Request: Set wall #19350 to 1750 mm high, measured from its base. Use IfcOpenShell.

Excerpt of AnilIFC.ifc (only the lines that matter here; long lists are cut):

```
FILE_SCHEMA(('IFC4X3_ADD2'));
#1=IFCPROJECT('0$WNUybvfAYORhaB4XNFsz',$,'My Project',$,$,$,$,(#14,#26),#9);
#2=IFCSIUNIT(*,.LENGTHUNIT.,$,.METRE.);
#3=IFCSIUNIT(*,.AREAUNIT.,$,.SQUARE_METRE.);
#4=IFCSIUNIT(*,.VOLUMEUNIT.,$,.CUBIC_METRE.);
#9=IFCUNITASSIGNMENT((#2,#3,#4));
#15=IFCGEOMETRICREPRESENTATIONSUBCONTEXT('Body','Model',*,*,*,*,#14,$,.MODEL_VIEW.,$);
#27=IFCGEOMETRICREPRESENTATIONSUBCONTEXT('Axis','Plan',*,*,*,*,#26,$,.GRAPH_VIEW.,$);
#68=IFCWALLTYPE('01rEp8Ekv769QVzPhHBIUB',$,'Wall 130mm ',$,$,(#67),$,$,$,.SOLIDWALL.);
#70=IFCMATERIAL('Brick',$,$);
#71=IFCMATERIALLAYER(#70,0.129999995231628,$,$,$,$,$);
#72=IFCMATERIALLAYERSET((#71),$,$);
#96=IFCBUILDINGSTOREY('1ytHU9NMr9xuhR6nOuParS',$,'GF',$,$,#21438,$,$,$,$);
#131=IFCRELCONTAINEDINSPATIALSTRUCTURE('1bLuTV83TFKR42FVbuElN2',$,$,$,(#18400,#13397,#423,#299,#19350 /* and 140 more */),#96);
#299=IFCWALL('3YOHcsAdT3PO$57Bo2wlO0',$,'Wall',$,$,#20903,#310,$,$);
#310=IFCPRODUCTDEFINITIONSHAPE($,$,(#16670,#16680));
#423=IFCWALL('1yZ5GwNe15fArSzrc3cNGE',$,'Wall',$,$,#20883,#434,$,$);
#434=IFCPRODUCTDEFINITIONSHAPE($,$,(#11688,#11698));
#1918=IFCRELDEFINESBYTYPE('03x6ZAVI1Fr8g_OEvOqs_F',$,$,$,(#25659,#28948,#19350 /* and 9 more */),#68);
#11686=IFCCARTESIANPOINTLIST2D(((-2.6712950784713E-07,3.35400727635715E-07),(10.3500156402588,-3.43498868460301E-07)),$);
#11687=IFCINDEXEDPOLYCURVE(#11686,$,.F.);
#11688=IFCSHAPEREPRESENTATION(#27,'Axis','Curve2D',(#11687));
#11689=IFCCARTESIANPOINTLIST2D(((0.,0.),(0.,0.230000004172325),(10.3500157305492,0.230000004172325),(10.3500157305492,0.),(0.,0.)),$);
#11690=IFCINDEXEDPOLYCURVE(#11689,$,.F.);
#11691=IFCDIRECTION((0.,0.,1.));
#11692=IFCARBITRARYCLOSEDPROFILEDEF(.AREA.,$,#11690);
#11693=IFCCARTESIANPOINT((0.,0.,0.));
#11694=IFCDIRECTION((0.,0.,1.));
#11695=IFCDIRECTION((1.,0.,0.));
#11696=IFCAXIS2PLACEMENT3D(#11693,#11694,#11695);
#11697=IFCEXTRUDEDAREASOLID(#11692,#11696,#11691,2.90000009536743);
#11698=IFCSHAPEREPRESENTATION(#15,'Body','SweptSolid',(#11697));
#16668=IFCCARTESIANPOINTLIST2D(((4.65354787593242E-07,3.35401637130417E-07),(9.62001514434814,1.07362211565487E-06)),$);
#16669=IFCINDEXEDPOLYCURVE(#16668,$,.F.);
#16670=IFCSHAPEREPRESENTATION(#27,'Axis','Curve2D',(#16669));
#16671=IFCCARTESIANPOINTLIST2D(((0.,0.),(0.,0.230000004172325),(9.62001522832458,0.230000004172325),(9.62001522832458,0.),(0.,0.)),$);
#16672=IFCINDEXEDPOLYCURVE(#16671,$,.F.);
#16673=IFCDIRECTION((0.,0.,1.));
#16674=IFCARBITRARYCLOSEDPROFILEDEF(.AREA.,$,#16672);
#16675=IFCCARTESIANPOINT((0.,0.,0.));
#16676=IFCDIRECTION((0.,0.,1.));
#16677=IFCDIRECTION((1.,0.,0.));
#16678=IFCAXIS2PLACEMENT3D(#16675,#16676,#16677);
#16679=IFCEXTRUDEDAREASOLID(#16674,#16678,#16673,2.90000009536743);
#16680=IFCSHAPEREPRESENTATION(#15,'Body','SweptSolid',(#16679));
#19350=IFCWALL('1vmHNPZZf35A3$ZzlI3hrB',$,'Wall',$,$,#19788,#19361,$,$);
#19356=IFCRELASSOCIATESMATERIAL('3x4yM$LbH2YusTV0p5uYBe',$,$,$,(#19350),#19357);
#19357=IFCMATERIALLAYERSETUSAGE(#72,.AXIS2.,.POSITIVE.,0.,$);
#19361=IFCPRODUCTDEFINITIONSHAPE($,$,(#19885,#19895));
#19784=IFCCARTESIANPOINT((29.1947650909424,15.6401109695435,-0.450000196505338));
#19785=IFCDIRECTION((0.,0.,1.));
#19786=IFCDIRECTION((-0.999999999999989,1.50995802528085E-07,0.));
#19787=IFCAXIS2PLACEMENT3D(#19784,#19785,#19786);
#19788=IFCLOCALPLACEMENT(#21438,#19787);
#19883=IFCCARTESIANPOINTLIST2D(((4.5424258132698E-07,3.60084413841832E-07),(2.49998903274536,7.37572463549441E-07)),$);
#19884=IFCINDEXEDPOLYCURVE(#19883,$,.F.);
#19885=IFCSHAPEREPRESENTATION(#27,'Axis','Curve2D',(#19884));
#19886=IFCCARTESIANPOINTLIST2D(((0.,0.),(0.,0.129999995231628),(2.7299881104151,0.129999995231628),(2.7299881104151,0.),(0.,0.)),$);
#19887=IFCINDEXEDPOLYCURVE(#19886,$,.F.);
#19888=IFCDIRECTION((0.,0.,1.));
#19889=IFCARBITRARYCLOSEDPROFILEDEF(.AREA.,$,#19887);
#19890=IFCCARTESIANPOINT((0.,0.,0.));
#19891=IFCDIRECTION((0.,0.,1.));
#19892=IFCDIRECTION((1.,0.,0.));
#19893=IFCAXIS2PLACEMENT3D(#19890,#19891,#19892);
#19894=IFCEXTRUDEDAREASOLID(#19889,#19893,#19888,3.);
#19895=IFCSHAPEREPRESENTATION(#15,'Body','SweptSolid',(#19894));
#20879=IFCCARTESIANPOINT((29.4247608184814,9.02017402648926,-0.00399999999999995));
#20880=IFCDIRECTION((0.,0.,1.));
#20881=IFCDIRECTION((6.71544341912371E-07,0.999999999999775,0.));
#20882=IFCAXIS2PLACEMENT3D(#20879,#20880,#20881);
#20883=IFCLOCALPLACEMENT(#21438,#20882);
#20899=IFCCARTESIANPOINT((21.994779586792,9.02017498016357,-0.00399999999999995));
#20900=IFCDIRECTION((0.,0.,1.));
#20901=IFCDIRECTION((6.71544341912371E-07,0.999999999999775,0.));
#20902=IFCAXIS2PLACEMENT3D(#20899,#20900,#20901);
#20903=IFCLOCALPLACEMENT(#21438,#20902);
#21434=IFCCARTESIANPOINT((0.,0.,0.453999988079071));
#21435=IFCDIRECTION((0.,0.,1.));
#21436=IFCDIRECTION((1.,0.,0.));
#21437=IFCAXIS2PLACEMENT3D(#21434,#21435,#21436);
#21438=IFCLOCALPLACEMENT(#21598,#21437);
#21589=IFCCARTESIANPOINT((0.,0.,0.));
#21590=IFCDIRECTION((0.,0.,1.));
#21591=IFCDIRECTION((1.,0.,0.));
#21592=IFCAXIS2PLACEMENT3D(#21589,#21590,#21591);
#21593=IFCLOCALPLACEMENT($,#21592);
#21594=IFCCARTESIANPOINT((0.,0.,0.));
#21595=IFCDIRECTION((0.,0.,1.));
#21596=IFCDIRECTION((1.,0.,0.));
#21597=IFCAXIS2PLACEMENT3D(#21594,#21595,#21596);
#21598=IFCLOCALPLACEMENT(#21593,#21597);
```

```python
import ifcopenshell
import ifcopenshell.geom
import ifcopenshell.util.representation
import ifcopenshell.util.shape
import ifcopenshell.util.unit

model = ifcopenshell.open("AnilIFC.ifc")
unit_scale = ifcopenshell.util.unit.calculate_unit_scale(model)
settings = ifcopenshell.geom.settings()


def volume(element):
    """Net volume in cubic metres, openings subtracted."""
    shape = ifcopenshell.geom.create_shape(settings, element)
    return ifcopenshell.util.shape.get_volume(shape.geometry)


wall = model.by_guid("1vmHNPZZf35A3$ZzlI3hrB")
before = volume(wall)

body = ifcopenshell.util.representation.get_representation(wall, "Model", "Body")
solid = body.Items[0]
old_height = solid.Depth
solid.Depth = 1.75 / unit_scale
after = volume(wall)

print(f"height {old_height:g} -> {solid.Depth:g}, volume {before:.3f} -> {after:.3f} m3")

model.write("AnilIFC_updated.ifc")
```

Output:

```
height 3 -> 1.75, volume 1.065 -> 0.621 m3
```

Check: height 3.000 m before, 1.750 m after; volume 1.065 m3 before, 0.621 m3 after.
